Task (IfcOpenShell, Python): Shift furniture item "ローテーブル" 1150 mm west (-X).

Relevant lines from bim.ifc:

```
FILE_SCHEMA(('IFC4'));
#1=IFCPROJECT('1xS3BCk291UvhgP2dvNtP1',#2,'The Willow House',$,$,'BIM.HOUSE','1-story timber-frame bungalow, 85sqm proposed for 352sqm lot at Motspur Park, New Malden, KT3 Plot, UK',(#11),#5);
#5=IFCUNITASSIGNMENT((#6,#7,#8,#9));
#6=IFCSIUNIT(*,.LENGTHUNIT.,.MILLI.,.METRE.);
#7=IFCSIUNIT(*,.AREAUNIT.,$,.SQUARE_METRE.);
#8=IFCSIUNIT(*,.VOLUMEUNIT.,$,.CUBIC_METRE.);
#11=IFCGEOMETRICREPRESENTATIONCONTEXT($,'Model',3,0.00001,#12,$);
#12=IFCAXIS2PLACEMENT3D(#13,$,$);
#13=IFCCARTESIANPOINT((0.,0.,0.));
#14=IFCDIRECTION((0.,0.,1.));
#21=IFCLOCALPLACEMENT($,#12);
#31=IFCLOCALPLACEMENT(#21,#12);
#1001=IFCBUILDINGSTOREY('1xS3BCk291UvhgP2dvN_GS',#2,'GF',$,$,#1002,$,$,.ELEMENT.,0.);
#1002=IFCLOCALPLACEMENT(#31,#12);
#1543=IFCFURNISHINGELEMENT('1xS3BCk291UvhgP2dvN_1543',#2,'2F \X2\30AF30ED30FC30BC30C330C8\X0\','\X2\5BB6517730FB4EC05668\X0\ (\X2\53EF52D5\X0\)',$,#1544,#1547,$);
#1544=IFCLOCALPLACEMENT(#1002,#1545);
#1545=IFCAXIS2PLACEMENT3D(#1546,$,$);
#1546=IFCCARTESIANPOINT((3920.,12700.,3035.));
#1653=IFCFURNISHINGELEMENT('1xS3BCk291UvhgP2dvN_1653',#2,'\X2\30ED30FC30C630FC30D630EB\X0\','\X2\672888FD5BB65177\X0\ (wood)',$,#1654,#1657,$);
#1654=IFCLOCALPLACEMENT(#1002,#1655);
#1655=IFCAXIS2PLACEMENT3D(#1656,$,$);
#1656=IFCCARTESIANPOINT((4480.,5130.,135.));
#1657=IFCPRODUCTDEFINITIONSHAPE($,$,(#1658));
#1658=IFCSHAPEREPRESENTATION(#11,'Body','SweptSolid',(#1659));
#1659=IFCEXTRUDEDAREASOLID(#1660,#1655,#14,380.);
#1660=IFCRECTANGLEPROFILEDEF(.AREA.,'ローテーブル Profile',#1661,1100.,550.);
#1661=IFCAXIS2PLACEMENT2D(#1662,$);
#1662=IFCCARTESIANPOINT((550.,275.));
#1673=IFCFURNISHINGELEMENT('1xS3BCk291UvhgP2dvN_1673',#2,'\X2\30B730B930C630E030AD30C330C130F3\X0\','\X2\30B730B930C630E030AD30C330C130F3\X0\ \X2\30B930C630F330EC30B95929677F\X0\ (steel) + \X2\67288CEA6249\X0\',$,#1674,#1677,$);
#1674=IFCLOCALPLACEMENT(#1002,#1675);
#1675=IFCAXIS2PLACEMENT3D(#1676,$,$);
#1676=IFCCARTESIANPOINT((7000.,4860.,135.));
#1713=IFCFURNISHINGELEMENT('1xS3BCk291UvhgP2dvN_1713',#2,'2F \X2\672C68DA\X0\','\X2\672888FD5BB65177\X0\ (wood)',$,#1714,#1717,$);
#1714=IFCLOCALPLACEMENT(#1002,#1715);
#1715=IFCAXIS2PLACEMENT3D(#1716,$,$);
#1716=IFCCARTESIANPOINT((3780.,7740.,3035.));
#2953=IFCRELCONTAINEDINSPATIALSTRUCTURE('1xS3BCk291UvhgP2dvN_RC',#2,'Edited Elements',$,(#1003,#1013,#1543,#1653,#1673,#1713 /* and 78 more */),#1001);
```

```python
import ifcopenshell
import ifcopenshell.api.geometry
import ifcopenshell.util.placement

model = ifcopenshell.open("bim.ifc")

item = model.by_id(1653)
matrix = ifcopenshell.util.placement.get_local_placement(item.ObjectPlacement)
matrix[0, 3] -= 1150.0
ifcopenshell.api.geometry.edit_object_placement(model, product=item, matrix=matrix, is_si=False)

print(ifcopenshell.util.placement.get_local_placement(item.ObjectPlacement).round(3) + 0.0)

model.write("bim_rev.ifc")
```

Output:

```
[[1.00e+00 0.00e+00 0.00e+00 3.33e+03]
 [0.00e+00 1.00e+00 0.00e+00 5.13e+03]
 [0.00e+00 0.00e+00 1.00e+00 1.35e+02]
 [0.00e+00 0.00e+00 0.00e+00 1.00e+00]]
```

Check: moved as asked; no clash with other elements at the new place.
